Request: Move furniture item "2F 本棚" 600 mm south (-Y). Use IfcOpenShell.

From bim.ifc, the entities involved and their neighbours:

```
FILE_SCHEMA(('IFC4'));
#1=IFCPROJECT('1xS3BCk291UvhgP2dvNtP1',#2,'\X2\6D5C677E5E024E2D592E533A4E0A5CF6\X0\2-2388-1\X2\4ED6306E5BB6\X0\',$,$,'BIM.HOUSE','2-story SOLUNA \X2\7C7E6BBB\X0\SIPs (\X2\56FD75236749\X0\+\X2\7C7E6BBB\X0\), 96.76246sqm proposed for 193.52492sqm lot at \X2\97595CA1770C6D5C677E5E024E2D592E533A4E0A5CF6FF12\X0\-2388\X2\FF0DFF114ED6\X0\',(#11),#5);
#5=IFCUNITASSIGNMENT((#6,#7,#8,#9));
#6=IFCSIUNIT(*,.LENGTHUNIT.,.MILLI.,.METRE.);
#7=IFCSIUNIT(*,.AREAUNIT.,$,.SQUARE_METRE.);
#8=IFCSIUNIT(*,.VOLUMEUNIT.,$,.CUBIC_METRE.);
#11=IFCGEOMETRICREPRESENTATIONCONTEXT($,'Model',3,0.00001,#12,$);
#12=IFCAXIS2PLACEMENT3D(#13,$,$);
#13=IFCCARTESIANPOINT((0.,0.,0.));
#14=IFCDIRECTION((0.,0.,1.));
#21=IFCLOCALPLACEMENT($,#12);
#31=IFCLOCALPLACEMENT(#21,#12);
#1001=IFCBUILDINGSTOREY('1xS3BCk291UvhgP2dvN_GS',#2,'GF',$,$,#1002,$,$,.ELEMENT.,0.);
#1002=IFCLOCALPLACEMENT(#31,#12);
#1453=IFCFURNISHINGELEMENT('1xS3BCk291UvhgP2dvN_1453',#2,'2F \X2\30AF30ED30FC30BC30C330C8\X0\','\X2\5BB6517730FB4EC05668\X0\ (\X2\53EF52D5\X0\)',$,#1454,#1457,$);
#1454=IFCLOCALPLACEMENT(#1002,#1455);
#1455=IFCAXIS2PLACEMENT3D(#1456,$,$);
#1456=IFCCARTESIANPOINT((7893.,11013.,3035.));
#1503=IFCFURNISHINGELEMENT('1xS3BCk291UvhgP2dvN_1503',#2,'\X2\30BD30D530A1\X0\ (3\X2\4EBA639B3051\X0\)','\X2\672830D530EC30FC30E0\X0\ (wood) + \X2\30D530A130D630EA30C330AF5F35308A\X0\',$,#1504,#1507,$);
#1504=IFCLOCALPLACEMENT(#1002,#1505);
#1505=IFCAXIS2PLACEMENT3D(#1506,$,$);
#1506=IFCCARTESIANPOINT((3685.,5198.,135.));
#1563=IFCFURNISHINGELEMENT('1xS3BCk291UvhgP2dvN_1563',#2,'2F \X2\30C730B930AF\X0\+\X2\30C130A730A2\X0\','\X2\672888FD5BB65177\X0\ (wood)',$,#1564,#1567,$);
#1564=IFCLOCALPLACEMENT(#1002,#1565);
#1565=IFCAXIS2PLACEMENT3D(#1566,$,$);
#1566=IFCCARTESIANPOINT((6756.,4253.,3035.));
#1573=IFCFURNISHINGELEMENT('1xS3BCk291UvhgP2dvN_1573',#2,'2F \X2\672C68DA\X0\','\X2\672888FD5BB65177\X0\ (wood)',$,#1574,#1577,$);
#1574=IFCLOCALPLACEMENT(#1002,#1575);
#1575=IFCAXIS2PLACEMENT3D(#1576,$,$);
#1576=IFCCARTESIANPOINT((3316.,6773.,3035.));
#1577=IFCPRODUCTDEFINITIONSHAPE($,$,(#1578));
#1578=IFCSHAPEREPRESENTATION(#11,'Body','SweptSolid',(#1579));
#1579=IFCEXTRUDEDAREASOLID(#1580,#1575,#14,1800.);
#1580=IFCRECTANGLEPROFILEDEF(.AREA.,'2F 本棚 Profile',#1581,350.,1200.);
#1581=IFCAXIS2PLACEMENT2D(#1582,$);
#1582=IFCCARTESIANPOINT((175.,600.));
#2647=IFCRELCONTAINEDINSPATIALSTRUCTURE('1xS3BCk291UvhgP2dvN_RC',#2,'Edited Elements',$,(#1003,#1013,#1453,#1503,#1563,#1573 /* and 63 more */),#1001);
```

```python
import ifcopenshell
import ifcopenshell.api.geometry
import ifcopenshell.util.placement

model = ifcopenshell.open("bim.ifc")

item = model.by_guid("1xS3BCk291UvhgP2dvN_1573")
matrix = ifcopenshell.util.placement.get_local_placement(item.ObjectPlacement)
matrix[1, 3] -= 600.0
ifcopenshell.api.geometry.edit_object_placement(model, product=item, matrix=matrix, is_si=False)

print(ifcopenshell.util.placement.get_local_placement(item.ObjectPlacement).round(3) + 0.0)

model.write("bim_v2.ifc")
```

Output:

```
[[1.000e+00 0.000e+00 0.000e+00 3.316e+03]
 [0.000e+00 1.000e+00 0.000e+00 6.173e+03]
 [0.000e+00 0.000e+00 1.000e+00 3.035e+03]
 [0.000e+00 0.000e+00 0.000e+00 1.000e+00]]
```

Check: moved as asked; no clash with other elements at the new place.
